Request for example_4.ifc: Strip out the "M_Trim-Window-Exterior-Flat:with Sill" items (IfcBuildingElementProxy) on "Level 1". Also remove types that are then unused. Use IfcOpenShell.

First a look at what the model holds.

```python
import ifcopenshell
import ifcopenshell.util.element

model = ifcopenshell.open("example_4.ifc")
print(model.schema)
storey = next(s for s in model.by_type("IfcBuildingStorey") if s.Name == "Level 1")
proxies = [e for e in ifcopenshell.util.element.get_decomposition(storey) if e.is_a("IfcBuildingElementProxy")]
seen = {}
for e in proxies:
    element_type = ifcopenshell.util.element.get_type(e)
    name = element_type.Name if element_type not in (None, e) else None
    seen[name] = seen.get(name, 0) + 1
for name, count in sorted(seen.items(), key=str):
    print(count, "x", name)
```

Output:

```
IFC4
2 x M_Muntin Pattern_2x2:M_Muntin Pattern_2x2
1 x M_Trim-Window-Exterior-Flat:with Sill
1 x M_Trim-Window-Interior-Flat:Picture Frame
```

```python
import ifcopenshell
import ifcopenshell.api.root
import ifcopenshell.util.element

model = ifcopenshell.open("example_4.ifc")

storey = next(s for s in model.by_type("IfcBuildingStorey") if s.Name == "Level 1")
proxies = [e for e in ifcopenshell.util.element.get_decomposition(storey) if e.is_a("IfcBuildingElementProxy")]
targets = [e for e in proxies if (t := ifcopenshell.util.element.get_type(e)) not in (None, e) and t.Name == "M_Trim-Window-Exterior-Flat:with Sill"]
types = {ifcopenshell.util.element.get_type(e) for e in targets} - {None, *targets}

for e in targets:
    ifcopenshell.api.root.remove_product(model, product=e)
print(len(targets), "removed")

unused = [t for t in types if not ifcopenshell.util.element.get_types(t)]
for t in unused:
    ifcopenshell.api.root.remove_product(model, product=t)
print(len(unused), "unused types removed")

model.write("example_4_v2.ifc")
```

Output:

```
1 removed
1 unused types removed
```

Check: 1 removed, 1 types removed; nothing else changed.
